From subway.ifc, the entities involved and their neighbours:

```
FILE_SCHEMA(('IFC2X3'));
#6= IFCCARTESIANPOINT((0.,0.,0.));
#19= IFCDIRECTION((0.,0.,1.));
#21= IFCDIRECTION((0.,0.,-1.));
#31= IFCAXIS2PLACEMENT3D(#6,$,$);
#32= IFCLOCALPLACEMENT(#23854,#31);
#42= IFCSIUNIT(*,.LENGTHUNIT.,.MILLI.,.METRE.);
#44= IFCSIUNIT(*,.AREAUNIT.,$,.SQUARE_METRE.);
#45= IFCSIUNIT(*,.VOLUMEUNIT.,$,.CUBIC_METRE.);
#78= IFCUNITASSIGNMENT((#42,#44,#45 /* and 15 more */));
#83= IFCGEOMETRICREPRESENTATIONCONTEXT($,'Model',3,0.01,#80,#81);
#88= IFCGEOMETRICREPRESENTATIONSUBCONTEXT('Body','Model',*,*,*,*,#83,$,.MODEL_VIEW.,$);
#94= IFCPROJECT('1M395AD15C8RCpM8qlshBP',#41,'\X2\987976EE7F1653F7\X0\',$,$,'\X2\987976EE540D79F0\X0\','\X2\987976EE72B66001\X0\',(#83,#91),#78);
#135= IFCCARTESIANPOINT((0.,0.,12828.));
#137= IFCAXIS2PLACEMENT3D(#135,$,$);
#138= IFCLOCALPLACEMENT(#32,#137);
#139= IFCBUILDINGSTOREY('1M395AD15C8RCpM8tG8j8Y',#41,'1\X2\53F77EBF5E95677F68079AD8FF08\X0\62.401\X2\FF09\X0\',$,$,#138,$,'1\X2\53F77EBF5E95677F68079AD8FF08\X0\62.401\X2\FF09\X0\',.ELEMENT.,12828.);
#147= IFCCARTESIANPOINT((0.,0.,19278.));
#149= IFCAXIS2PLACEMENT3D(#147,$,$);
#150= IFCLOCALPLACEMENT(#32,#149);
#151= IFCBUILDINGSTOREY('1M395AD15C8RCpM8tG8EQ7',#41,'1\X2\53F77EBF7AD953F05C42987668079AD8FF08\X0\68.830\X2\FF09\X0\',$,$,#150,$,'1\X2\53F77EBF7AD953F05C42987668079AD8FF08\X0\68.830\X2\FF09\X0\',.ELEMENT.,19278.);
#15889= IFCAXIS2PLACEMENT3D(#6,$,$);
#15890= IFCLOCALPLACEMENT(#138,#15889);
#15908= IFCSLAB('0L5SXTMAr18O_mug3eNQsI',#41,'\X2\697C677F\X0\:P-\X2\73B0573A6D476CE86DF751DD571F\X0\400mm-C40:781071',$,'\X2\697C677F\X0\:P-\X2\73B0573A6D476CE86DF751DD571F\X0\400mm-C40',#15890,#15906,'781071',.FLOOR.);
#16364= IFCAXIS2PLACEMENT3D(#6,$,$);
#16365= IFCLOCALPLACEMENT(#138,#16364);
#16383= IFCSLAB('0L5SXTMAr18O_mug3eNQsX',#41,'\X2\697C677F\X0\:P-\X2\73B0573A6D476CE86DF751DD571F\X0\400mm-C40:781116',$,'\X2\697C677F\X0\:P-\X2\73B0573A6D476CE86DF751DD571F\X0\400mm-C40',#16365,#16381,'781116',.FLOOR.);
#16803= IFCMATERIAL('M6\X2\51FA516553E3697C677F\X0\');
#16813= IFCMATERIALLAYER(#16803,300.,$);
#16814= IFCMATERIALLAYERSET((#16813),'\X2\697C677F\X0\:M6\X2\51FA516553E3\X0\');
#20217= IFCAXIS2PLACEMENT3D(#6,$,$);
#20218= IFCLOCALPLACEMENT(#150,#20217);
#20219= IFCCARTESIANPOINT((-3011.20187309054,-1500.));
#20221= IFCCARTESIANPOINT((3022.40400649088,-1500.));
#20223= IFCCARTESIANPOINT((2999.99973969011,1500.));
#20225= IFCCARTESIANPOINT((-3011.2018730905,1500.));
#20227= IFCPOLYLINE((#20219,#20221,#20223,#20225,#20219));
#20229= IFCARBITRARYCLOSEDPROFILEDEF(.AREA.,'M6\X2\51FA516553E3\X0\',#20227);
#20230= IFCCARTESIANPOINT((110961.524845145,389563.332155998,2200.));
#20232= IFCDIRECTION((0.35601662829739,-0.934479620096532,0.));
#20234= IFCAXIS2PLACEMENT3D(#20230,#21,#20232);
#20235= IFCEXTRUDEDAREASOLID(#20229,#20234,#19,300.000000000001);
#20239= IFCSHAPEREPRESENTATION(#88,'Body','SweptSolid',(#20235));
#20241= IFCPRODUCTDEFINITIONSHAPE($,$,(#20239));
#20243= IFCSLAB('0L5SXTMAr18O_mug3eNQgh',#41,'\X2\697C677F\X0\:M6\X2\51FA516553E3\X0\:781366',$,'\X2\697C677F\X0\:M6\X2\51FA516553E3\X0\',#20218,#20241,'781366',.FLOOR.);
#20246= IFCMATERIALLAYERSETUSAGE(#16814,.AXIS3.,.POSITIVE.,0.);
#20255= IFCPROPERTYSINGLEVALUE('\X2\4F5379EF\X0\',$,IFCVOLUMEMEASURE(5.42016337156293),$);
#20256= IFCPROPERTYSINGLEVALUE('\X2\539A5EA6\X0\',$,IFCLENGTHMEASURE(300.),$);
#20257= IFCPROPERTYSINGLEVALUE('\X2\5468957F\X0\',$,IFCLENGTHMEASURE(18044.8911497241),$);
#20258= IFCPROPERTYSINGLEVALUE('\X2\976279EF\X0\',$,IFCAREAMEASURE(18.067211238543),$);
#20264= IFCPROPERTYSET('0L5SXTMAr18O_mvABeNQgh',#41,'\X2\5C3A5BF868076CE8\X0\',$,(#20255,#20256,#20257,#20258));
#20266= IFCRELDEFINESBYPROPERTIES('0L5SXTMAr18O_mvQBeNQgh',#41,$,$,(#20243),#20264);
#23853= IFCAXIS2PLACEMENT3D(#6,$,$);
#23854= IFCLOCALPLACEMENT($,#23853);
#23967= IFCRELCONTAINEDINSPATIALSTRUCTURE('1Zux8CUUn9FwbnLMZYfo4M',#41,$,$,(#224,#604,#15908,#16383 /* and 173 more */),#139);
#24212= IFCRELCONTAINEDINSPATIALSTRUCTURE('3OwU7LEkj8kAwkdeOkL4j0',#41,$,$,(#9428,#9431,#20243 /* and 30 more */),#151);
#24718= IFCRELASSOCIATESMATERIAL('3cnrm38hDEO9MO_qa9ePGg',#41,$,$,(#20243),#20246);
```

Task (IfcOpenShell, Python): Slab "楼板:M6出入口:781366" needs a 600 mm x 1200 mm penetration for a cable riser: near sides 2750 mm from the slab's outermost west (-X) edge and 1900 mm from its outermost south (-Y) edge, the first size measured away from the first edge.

```python
import numpy as np
import ifcopenshell
import ifcopenshell.api.feature
import ifcopenshell.api.geometry
import ifcopenshell.api.pset
import ifcopenshell.api.root
import ifcopenshell.geom
import ifcopenshell.util.element
import ifcopenshell.util.placement
import ifcopenshell.util.representation
import ifcopenshell.util.shape
import ifcopenshell.util.unit

model = ifcopenshell.open("subway.ifc")
unit_scale = ifcopenshell.util.unit.calculate_unit_scale(model)
area_scale = ifcopenshell.util.unit.calculate_unit_scale(model, "AREAUNIT")
volume_scale = ifcopenshell.util.unit.calculate_unit_scale(model, "VOLUMEUNIT")
settings = ifcopenshell.geom.settings()


def volume(element):
    """Net volume in cubic metres, openings subtracted."""
    shape = ifcopenshell.geom.create_shape(settings, element)
    return ifcopenshell.util.shape.get_volume(shape.geometry)


slab = model.by_guid("0L5SXTMAr18O_mug3eNQgh")
before = volume(slab)

# Extent in the slab's own axes, in metres. The edges named are its -X and -Y sides.
slab_shape = ifcopenshell.geom.create_shape(settings, slab)
vertices = ifcopenshell.util.shape.get_vertices(slab_shape.geometry)
x_min, y_min, bottom = vertices.min(axis=0)
top = vertices[:, 2].max()

opening = ifcopenshell.api.root.create_entity(model, ifc_class="IfcOpeningElement", name="Cable riser opening")
context = ifcopenshell.util.representation.get_context(model, "Model", "Body", "MODEL_VIEW")
width, depth = 0.6, 1.2
outline = [(0.0, 0.0), (width, 0.0), (width, depth), (0.0, depth), (0.0, 0.0)]
# Overshoot both faces by 50 mm so the cut is clean.
shape = ifcopenshell.api.geometry.add_slab_representation(
    model, context=context, depth=top - bottom + 0.1, polyline=outline
)
ifcopenshell.api.geometry.assign_representation(model, product=opening, representation=shape)

matrix = ifcopenshell.util.placement.get_local_placement(slab.ObjectPlacement)
matrix[:, 3] = matrix @ np.append(np.array([x_min + 2.75, y_min + 1.9, bottom - 0.05]) / unit_scale, 1.0)
ifcopenshell.api.geometry.edit_object_placement(model, product=opening, matrix=matrix, is_si=False)
ifcopenshell.api.feature.add_feature(model, feature=opening, element=slab)

after = volume(slab)

# Update the slab's stored quantities.
pset = model.by_id(ifcopenshell.util.element.get_pset(slab, "尺寸标注", should_inherit=False)["id"])
ifcopenshell.api.pset.edit_pset(model, pset=pset, properties={
    "体积": model.create_entity("IfcVolumeMeasure", after / volume_scale),
    "面积": model.create_entity("IfcAreaMeasure", after / (top - bottom) / area_scale),
})

print(f"slab volume {before:.3f} -> {after:.3f} m3")

model.write("subway_updated.ifc")
```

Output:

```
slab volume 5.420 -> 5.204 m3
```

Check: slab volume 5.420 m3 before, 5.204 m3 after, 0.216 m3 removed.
